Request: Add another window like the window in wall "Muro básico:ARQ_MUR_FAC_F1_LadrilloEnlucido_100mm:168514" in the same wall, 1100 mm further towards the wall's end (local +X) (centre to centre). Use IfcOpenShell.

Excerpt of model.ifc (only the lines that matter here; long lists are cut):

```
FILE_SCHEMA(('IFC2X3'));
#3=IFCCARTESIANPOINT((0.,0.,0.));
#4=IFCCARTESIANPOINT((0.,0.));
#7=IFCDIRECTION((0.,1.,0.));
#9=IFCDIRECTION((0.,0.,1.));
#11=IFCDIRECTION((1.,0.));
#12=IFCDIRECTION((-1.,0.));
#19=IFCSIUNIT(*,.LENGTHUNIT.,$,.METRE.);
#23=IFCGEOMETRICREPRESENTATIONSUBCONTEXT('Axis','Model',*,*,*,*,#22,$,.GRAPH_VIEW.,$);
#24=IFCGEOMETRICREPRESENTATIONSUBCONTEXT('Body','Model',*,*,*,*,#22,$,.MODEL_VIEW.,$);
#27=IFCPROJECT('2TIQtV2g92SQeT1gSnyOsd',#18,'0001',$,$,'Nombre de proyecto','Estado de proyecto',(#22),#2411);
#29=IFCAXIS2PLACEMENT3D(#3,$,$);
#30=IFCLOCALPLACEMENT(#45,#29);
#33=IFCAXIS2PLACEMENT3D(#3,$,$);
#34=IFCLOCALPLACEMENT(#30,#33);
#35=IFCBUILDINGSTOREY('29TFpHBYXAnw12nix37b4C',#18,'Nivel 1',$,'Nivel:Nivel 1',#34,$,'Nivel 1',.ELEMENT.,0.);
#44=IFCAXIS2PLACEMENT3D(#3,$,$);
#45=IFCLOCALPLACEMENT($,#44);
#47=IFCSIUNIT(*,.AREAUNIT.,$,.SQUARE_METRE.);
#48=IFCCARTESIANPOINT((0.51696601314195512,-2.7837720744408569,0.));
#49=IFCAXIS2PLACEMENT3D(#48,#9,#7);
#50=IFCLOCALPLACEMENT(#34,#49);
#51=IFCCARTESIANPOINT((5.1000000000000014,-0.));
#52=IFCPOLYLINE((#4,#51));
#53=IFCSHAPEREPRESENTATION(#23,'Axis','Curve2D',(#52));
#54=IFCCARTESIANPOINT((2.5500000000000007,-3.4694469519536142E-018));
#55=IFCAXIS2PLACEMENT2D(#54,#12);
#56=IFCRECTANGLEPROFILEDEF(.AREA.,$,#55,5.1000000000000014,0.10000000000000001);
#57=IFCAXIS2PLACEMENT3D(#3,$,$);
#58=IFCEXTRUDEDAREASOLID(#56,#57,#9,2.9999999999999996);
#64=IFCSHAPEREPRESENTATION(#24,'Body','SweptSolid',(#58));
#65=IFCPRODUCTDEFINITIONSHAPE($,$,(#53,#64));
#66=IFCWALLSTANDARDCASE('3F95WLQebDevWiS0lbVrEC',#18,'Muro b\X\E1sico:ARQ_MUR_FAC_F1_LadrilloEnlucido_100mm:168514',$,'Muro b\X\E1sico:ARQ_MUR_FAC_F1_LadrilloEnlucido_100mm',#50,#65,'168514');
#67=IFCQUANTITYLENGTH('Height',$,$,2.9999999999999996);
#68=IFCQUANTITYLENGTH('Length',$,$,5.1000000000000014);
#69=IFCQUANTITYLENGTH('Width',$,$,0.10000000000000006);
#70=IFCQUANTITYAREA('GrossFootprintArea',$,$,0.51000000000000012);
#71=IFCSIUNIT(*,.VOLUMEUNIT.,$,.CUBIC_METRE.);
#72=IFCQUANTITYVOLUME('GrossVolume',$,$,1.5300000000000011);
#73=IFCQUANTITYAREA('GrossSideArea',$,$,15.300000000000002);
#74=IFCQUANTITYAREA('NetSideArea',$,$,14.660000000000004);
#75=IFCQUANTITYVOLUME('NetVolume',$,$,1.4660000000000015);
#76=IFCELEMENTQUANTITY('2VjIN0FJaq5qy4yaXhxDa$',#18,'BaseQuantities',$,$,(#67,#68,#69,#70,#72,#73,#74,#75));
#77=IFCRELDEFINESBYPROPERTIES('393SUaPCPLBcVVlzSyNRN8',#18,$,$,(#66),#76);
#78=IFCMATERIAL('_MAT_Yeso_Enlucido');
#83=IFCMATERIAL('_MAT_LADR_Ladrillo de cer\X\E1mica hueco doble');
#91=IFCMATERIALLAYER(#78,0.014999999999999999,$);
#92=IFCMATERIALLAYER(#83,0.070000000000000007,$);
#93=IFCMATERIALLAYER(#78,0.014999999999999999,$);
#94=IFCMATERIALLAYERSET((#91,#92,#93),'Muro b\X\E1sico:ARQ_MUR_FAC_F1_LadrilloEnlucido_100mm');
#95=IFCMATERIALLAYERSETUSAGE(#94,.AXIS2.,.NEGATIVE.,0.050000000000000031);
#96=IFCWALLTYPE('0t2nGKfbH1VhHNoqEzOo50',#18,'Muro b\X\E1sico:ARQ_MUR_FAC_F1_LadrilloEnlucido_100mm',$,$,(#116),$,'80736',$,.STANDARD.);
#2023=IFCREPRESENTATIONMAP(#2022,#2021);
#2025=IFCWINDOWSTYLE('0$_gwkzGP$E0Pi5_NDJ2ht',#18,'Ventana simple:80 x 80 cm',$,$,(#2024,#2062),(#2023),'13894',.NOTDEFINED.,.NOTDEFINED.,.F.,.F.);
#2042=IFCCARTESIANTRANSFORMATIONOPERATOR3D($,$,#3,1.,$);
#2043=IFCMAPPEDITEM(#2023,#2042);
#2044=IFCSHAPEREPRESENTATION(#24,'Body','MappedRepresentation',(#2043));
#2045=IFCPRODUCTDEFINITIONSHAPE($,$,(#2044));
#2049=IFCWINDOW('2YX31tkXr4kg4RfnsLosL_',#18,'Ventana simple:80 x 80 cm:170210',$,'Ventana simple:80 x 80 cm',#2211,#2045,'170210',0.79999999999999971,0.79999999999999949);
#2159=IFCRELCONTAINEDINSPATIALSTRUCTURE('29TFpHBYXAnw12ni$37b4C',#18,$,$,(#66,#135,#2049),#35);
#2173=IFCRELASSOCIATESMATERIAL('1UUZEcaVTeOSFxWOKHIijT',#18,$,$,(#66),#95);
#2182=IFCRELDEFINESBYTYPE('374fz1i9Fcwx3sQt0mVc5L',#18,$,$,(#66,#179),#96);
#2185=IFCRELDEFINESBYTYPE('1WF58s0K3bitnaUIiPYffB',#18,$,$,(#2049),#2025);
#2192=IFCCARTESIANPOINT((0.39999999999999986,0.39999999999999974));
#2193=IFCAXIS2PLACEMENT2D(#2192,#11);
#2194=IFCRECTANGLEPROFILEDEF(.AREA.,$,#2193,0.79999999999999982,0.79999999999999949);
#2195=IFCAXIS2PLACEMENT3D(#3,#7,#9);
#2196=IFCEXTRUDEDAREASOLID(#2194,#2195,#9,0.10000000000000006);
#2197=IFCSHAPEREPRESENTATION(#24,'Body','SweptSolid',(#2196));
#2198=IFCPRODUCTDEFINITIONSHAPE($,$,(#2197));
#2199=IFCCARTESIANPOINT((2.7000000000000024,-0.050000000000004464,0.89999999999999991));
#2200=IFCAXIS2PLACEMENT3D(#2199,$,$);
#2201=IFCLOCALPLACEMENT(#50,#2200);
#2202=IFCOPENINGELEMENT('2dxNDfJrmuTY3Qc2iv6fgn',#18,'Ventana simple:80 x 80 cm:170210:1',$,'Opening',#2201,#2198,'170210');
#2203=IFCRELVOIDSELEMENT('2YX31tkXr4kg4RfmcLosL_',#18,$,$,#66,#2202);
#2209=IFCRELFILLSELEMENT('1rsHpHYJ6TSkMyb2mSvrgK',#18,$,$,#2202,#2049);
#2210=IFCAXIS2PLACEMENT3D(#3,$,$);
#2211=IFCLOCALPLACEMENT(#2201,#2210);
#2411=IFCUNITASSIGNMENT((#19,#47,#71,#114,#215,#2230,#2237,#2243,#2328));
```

```python
import ifcopenshell
import ifcopenshell.api.feature
import ifcopenshell.api.geometry
import ifcopenshell.api.pset
import ifcopenshell.api.root
import ifcopenshell.geom
import ifcopenshell.util.element
import ifcopenshell.util.placement
import ifcopenshell.util.shape
import ifcopenshell.util.unit

model = ifcopenshell.open("model.ifc")
unit_scale = ifcopenshell.util.unit.calculate_unit_scale(model)
area_scale = ifcopenshell.util.unit.calculate_unit_scale(model, "AREAUNIT")
volume_scale = ifcopenshell.util.unit.calculate_unit_scale(model, "VOLUMEUNIT")
settings = ifcopenshell.geom.settings()


def volume(element):
    """Net volume in cubic metres, openings subtracted."""
    shape = ifcopenshell.geom.create_shape(settings, element)
    return ifcopenshell.util.shape.get_volume(shape.geometry)


def reuse_history(source, copy):
    """copy_class also copies each property set's owner history, people and application; keep the originals."""
    for rel in copy.IsDefinedBy:
        if rel.is_a("IfcRelDefinesByProperties") and (history := rel.RelatingPropertyDefinition.OwnerHistory):
            rel.RelatingPropertyDefinition.OwnerHistory = source.OwnerHistory
            ifcopenshell.util.element.remove_deep2(model, history)


window = model.by_id(2049)
opening = window.FillsVoids[0].RelatingOpeningElement
wall = opening.VoidsElements[0].RelatingBuildingElement
before = volume(wall)
shift = ifcopenshell.util.placement.get_local_placement(wall.ObjectPlacement)[:3, 0] * 1.1 / unit_scale

# copy_class copies the void relationship, type, container and properties, but no geometry.
new_opening = ifcopenshell.api.root.copy_class(model, product=opening)
new_opening.Representation = ifcopenshell.util.element.copy_deep(
    model, opening.Representation, exclude=["IfcGeometricRepresentationContext", "IfcRepresentationMap"]
)
new_opening.Name = "Ventana simple:80 x 80 cm"
new_opening.Tag = None
reuse_history(opening, new_opening)
new_window = ifcopenshell.api.root.copy_class(model, product=window)
new_window.Representation = ifcopenshell.util.element.copy_deep(
    model, window.Representation, exclude=["IfcGeometricRepresentationContext", "IfcRepresentationMap"]
)
new_window.Name = "Ventana simple:80 x 80 cm"
new_window.Tag = None
reuse_history(window, new_window)
fills = ifcopenshell.api.feature.add_filling(model, opening=new_opening, element=new_window)
fills.OwnerHistory = new_window.OwnerHistory  # required in IFC2X3

for old, new in ((opening, new_opening), (window, new_window)):
    matrix = ifcopenshell.util.placement.get_local_placement(old.ObjectPlacement)
    matrix[:3, 3] += shift
    ifcopenshell.api.geometry.edit_object_placement(model, product=new, matrix=matrix, is_si=False)

after = volume(wall)
thickness = 0.1  # wall thickness in metres

# Update the wall's stored quantities.
qto = model.by_id(ifcopenshell.util.element.get_pset(wall, "BaseQuantities", should_inherit=False)["id"])
ifcopenshell.api.pset.edit_qto(model, qto=qto, properties={
    "NetSideArea": after / thickness / area_scale,
    "NetVolume": after / volume_scale,
})

print(f"wall volume {before:.3f} -> {after:.3f} m3")

model.write("model-out.ifc")
```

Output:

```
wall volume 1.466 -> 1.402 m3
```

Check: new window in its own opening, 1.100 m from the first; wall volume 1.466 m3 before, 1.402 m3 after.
